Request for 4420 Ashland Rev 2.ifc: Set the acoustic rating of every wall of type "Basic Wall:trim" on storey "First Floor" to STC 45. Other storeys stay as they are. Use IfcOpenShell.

First a look at what the model holds.

```python
import ifcopenshell
import ifcopenshell.util.element

model = ifcopenshell.open("4420 Ashland Rev 2.ifc")
print(model.schema)
storey = next(s for s in model.by_type("IfcBuildingStorey") if s.Name == "First Floor")
walls = [e for e in ifcopenshell.util.element.get_decomposition(storey) if e.is_a("IfcWall")]
seen = {}
for e in walls:
    element_type = ifcopenshell.util.element.get_type(e)
    key = (element_type.Name if element_type != e and element_type else None, ifcopenshell.util.element.get_pset(e, "Pset_WallCommon", "AcousticRating"))
    seen[key] = seen.get(key, 0) + 1
for (name, value), count in sorted(seen.items(), key=str):
    print(count, "x", name, "|", value)
```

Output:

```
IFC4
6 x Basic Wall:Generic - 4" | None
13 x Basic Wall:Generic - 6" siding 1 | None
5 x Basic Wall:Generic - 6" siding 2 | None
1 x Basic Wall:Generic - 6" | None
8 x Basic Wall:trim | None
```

```python
import ifcopenshell
import ifcopenshell.api.pset
import ifcopenshell.util.element

model = ifcopenshell.open("4420 Ashland Rev 2.ifc")

storey = next(s for s in model.by_type("IfcBuildingStorey") if s.Name == "First Floor")
walls = [e for e in ifcopenshell.util.element.get_decomposition(storey) if e.is_a("IfcWall")]

count = 0
for e in walls:
    element_type = ifcopenshell.util.element.get_type(e)
    if element_type in (None, e) or element_type.Name != "Basic Wall:trim":
        continue
    # add_pset returns the element's existing set when there is one.
    pset = ifcopenshell.api.pset.add_pset(model, product=e, name="Pset_WallCommon")
    ifcopenshell.api.pset.edit_pset(model, pset=pset, properties={"AcousticRating": "STC 45"})
    count += 1

print(count, "walls updated")

model.write("4420 Ashland Rev 2_rev.ifc")
```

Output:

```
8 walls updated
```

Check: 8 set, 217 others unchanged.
